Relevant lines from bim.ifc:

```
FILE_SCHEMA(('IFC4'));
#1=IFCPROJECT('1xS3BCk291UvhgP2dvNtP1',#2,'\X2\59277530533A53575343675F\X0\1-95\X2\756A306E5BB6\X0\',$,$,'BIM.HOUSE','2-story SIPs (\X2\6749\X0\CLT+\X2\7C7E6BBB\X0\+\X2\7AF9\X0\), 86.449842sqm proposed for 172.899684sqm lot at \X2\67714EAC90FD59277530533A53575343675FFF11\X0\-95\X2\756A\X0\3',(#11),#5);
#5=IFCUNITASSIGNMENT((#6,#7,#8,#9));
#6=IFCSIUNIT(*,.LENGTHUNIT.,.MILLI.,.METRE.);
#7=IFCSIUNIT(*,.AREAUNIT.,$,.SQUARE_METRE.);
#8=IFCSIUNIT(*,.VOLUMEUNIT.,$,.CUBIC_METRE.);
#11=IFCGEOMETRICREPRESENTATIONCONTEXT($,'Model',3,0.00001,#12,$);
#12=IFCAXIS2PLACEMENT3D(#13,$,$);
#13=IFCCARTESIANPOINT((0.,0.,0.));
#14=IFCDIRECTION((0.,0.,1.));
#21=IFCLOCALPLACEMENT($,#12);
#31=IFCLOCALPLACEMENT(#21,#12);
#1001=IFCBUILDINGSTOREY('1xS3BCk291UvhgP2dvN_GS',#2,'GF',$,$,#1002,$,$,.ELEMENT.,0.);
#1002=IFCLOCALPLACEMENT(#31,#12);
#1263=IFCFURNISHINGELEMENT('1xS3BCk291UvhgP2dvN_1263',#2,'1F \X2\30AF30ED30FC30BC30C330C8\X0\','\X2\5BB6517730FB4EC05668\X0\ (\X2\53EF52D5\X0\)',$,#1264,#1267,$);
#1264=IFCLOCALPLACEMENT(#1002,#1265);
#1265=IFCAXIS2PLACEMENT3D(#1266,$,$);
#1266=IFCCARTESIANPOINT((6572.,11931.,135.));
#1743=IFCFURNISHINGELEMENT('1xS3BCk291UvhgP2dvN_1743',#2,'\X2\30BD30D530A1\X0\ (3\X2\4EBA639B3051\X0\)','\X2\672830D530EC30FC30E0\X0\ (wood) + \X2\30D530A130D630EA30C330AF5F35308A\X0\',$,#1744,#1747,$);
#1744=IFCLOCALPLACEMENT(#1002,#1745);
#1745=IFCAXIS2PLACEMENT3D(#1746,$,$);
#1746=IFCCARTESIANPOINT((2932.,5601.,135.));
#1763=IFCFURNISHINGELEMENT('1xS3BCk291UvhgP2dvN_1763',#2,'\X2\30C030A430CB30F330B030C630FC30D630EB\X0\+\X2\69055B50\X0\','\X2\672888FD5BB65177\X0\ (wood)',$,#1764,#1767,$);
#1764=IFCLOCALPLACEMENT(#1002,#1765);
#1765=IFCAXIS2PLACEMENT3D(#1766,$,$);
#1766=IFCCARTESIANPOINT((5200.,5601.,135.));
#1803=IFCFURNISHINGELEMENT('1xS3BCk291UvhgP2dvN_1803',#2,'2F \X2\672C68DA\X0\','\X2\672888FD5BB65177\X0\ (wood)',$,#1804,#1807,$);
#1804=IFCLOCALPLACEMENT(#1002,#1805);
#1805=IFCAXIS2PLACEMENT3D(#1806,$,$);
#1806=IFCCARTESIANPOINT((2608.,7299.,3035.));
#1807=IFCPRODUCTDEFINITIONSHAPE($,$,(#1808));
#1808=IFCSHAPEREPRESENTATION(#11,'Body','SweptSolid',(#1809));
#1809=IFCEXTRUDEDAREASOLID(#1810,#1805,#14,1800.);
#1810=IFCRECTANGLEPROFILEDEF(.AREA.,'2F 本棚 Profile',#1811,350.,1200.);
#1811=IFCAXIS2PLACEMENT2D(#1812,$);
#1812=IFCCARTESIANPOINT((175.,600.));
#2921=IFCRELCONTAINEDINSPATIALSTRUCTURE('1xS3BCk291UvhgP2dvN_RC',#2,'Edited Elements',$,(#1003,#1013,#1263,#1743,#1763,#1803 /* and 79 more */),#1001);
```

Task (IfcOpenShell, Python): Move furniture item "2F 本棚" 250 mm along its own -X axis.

```python
import ifcopenshell
import ifcopenshell.api.geometry
import ifcopenshell.util.placement
import ifcopenshell.util.unit

model = ifcopenshell.open("bim.ifc")
unit_scale = ifcopenshell.util.unit.calculate_unit_scale(model)

item = model.by_id(1803)
matrix = ifcopenshell.util.placement.get_local_placement(item.ObjectPlacement)
matrix[:3, 3] -= matrix[:3, 0] * 0.25 / unit_scale
ifcopenshell.api.geometry.edit_object_placement(model, product=item, matrix=matrix, is_si=False)

print(ifcopenshell.util.placement.get_local_placement(item.ObjectPlacement).round(3) + 0.0)

model.write("bim_updated.ifc")
```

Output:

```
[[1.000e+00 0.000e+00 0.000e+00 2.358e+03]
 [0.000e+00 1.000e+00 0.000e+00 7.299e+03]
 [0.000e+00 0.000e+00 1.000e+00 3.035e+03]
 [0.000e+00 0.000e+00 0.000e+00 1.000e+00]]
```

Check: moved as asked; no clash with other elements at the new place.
